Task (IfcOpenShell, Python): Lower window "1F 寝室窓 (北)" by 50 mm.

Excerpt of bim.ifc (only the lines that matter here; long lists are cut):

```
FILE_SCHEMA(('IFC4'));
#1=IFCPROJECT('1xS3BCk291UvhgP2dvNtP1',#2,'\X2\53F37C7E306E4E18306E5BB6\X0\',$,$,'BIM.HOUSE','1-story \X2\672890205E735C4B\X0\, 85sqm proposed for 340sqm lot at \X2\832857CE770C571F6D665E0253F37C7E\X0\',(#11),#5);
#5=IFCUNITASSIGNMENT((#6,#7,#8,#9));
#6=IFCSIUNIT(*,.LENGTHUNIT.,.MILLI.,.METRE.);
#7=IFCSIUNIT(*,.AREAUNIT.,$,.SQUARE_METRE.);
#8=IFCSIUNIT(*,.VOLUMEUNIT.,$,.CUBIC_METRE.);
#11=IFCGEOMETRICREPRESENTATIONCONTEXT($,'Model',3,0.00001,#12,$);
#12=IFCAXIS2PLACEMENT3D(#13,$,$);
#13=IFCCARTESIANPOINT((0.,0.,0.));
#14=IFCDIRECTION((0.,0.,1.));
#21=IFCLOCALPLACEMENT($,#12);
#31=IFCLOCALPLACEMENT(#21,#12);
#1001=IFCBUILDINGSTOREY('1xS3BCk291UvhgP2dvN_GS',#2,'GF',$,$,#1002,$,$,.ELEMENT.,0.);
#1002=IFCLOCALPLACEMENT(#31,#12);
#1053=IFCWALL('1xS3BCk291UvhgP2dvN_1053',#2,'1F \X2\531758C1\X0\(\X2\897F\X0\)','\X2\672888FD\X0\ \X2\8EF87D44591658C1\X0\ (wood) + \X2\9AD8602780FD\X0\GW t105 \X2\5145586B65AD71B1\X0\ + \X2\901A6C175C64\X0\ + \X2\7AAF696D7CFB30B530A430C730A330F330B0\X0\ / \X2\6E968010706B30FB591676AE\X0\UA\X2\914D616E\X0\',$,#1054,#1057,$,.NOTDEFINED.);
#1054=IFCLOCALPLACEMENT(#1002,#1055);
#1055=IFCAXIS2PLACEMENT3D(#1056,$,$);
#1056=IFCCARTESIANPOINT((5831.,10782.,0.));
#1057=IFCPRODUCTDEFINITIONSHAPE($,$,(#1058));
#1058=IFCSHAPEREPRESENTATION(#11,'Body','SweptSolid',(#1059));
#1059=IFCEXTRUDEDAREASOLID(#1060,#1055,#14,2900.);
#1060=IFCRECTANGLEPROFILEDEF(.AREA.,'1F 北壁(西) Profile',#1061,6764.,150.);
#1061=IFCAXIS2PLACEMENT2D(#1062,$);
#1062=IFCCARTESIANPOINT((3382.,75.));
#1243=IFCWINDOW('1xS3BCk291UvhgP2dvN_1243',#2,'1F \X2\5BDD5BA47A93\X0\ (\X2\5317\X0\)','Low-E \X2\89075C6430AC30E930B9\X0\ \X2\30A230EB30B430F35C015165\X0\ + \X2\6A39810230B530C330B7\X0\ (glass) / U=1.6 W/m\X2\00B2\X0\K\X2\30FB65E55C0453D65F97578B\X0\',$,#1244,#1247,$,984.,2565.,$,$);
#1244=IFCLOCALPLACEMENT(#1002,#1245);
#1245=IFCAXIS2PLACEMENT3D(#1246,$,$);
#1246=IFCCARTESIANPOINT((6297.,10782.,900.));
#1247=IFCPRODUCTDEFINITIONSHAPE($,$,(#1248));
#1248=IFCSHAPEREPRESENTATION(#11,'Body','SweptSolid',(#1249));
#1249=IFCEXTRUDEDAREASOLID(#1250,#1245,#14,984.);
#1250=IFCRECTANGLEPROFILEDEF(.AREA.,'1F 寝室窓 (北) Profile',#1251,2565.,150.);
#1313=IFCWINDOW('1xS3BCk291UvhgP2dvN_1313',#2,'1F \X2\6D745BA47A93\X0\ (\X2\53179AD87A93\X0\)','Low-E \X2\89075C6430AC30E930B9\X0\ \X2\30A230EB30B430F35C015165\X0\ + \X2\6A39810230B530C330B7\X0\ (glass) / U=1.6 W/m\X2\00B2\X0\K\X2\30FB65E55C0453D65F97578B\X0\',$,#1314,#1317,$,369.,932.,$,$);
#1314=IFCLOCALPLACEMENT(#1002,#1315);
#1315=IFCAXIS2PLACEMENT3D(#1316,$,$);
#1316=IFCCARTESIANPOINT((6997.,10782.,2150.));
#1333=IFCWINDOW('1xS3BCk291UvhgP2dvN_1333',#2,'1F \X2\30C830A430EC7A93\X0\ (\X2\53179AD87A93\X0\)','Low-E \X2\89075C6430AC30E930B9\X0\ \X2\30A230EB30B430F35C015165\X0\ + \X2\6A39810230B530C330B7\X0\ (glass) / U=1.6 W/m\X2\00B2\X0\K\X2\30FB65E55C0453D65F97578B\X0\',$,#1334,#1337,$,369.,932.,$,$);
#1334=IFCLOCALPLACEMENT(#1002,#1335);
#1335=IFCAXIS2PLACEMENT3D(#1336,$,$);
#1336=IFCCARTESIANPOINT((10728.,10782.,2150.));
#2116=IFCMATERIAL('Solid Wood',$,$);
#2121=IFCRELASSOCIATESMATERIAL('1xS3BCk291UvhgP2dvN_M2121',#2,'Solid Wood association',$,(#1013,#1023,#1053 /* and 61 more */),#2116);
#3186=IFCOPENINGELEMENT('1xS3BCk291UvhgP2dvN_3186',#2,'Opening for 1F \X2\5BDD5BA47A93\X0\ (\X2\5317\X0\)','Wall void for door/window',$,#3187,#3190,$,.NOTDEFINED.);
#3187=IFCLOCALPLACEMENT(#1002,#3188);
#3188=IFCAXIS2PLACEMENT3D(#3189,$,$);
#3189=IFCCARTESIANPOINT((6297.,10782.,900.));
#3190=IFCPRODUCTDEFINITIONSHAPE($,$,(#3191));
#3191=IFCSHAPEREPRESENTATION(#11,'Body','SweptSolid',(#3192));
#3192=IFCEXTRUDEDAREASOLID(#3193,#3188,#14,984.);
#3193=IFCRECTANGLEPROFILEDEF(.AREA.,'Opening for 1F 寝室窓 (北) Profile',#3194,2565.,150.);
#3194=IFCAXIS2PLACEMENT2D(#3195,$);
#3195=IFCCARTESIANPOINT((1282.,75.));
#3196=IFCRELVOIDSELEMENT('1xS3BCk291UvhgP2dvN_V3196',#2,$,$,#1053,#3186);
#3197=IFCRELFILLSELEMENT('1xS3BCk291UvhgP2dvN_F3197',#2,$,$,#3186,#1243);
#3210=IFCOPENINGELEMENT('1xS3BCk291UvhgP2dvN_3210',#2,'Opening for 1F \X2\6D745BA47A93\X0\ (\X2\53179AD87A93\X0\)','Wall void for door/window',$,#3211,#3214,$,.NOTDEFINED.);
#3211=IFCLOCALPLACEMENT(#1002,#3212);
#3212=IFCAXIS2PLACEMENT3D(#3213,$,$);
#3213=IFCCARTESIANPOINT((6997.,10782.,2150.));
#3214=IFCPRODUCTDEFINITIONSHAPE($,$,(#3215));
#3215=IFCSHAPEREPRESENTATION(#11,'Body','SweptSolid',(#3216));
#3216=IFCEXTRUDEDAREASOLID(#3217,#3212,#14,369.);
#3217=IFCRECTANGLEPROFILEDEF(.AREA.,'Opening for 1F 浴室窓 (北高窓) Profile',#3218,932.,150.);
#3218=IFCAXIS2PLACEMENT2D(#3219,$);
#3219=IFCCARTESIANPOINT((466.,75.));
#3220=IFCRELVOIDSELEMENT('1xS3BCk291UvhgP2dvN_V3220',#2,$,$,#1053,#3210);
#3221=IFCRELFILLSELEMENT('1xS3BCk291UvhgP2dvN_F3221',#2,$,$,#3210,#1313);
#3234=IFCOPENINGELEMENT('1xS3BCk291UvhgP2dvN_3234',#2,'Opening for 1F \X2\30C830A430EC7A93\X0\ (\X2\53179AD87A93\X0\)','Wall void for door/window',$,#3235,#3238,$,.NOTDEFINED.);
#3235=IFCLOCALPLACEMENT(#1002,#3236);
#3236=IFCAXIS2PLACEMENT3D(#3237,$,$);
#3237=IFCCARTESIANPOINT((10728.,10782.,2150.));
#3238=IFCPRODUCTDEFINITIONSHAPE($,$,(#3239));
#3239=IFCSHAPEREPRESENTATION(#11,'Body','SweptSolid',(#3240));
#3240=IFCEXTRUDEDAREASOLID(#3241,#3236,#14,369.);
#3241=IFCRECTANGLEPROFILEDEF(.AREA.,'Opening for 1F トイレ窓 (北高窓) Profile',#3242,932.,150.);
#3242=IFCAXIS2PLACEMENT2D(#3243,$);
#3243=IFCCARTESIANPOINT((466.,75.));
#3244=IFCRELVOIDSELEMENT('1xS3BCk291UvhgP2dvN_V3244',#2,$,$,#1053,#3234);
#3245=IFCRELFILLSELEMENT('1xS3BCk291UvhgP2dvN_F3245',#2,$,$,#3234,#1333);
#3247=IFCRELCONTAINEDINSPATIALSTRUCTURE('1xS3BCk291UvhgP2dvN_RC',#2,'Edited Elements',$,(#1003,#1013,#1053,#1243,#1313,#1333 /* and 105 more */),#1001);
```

```python
import numpy as np
import ifcopenshell
import ifcopenshell.api.geometry
import ifcopenshell.util.placement
import ifcopenshell.util.unit

model = ifcopenshell.open("bim.ifc")
unit_scale = ifcopenshell.util.unit.calculate_unit_scale(model)

window = model.by_guid("1xS3BCk291UvhgP2dvN_1243")
opening = window.FillsVoids[0].RelatingOpeningElement
dz = -0.05 / unit_scale

shift = np.array([0.0, 0.0, dz])
# The window is not placed relative to its opening, so move both.
for product in (opening, window):
    matrix = ifcopenshell.util.placement.get_local_placement(product.ObjectPlacement)
    matrix[:3, 3] += shift
    ifcopenshell.api.geometry.edit_object_placement(model, product=product, matrix=matrix, is_si=False)

print(f"moved by {dz * unit_scale:+.3f} m")

model.write("bim_edited.ifc")
```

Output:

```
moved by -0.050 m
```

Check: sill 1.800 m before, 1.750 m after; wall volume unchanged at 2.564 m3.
